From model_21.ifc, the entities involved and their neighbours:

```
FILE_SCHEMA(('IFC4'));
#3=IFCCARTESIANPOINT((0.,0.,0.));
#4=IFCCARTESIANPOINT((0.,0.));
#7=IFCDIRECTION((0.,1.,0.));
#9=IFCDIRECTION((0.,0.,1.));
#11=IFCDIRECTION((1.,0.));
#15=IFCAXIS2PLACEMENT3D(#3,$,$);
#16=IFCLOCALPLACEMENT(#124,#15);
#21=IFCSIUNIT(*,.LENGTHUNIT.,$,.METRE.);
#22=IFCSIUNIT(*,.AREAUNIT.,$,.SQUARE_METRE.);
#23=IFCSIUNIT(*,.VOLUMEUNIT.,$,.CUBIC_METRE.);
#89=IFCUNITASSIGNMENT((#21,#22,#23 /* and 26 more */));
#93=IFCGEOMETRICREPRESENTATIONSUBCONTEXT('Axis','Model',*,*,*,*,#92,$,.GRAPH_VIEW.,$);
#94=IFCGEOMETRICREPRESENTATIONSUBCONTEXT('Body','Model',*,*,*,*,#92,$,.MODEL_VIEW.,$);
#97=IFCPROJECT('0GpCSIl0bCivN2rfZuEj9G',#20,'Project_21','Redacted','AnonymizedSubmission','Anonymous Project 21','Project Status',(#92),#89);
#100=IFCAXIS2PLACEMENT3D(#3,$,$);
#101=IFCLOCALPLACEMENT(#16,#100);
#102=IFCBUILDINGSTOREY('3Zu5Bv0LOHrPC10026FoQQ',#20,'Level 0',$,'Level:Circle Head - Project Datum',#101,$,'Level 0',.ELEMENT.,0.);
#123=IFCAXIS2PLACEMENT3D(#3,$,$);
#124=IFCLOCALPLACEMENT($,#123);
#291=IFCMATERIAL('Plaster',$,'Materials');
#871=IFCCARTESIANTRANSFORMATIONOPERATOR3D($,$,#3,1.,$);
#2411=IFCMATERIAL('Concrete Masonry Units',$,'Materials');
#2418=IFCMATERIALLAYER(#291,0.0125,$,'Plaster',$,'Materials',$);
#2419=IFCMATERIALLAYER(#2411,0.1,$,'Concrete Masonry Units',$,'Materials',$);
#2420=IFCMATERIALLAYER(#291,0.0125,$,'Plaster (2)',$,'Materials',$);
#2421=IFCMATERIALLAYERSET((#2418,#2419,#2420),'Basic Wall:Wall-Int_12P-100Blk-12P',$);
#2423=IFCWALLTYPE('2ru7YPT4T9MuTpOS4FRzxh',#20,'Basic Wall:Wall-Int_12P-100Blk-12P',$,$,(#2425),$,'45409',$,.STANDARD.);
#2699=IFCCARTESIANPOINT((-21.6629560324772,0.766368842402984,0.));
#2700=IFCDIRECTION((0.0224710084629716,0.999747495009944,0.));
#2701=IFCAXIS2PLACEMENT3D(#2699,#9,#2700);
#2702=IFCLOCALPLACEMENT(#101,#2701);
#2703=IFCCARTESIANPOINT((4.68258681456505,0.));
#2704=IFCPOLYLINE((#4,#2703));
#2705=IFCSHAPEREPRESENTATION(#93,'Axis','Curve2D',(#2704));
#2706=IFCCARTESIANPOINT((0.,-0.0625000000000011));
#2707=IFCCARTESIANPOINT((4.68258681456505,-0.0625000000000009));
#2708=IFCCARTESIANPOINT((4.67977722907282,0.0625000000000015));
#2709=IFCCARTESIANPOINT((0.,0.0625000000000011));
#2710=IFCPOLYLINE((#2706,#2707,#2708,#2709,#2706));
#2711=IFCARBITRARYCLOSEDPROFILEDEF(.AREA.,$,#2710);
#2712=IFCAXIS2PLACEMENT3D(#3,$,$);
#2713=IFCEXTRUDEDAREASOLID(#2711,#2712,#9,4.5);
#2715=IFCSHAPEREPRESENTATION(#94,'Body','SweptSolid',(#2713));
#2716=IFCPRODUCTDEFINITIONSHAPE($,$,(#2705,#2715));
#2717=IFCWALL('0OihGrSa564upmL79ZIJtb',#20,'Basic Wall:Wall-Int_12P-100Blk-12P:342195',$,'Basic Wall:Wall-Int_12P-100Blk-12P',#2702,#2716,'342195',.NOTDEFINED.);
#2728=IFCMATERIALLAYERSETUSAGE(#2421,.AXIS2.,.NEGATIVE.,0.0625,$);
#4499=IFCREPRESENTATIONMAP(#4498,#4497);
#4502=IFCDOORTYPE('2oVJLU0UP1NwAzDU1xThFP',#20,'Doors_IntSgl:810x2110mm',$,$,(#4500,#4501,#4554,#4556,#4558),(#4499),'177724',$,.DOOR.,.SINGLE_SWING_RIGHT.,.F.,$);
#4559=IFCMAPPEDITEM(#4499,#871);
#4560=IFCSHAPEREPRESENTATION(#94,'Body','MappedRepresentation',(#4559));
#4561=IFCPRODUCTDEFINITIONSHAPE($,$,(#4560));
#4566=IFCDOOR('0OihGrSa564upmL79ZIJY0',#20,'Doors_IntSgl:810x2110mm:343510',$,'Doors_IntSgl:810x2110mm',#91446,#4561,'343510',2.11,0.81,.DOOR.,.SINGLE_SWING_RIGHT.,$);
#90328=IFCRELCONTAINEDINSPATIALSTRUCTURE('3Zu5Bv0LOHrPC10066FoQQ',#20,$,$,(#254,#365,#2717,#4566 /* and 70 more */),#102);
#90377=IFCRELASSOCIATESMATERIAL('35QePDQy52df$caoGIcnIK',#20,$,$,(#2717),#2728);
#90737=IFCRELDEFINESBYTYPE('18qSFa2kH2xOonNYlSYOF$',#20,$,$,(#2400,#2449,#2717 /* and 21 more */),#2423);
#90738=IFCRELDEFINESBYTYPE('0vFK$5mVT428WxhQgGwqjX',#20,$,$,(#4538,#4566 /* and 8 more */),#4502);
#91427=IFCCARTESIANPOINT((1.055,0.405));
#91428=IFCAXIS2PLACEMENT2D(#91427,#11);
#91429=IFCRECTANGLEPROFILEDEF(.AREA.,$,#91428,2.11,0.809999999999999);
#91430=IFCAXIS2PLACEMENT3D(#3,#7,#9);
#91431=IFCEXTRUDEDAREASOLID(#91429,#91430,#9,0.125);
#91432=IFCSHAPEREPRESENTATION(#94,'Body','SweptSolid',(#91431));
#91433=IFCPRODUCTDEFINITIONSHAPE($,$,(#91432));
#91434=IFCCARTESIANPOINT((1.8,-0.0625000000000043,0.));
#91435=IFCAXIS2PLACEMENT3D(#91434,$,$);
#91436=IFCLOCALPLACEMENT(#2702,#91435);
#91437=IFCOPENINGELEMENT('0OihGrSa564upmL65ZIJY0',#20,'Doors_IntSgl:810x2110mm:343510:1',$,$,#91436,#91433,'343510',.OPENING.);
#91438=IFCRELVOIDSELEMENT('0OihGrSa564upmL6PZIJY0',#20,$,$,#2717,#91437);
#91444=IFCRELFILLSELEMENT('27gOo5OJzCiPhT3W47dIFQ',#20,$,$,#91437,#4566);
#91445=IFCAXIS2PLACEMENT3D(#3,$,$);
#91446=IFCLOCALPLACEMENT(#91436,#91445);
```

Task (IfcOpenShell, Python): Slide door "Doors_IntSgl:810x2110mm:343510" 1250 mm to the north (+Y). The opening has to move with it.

```python
import ifcopenshell
import ifcopenshell.api.geometry
import ifcopenshell.util.placement

model = ifcopenshell.open("model_21.ifc")

door = model.by_id(4566)
opening = door.FillsVoids[0].RelatingOpeningElement
wall = opening.VoidsElements[0].RelatingBuildingElement

wall_matrix = ifcopenshell.util.placement.get_local_placement(wall.ObjectPlacement)
shift = wall_matrix[:3, 0] * 1.25
before = ifcopenshell.util.placement.get_local_placement(door.ObjectPlacement)[:3, 3].copy()

# The door is placed relative to its opening, so it follows when the opening moves.
matrix = ifcopenshell.util.placement.get_local_placement(opening.ObjectPlacement)
matrix[:3, 3] += shift
ifcopenshell.api.geometry.edit_object_placement(
    model, product=opening, matrix=matrix, is_si=False, should_transform_children=True
)

after = ifcopenshell.util.placement.get_local_placement(door.ObjectPlacement)[:3, 3]
print("door moved by", (after - before).round(3) + 0.0)

model.write("model_21_edited.ifc")
```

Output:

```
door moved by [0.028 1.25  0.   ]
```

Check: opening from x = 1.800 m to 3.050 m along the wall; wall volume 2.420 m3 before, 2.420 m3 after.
